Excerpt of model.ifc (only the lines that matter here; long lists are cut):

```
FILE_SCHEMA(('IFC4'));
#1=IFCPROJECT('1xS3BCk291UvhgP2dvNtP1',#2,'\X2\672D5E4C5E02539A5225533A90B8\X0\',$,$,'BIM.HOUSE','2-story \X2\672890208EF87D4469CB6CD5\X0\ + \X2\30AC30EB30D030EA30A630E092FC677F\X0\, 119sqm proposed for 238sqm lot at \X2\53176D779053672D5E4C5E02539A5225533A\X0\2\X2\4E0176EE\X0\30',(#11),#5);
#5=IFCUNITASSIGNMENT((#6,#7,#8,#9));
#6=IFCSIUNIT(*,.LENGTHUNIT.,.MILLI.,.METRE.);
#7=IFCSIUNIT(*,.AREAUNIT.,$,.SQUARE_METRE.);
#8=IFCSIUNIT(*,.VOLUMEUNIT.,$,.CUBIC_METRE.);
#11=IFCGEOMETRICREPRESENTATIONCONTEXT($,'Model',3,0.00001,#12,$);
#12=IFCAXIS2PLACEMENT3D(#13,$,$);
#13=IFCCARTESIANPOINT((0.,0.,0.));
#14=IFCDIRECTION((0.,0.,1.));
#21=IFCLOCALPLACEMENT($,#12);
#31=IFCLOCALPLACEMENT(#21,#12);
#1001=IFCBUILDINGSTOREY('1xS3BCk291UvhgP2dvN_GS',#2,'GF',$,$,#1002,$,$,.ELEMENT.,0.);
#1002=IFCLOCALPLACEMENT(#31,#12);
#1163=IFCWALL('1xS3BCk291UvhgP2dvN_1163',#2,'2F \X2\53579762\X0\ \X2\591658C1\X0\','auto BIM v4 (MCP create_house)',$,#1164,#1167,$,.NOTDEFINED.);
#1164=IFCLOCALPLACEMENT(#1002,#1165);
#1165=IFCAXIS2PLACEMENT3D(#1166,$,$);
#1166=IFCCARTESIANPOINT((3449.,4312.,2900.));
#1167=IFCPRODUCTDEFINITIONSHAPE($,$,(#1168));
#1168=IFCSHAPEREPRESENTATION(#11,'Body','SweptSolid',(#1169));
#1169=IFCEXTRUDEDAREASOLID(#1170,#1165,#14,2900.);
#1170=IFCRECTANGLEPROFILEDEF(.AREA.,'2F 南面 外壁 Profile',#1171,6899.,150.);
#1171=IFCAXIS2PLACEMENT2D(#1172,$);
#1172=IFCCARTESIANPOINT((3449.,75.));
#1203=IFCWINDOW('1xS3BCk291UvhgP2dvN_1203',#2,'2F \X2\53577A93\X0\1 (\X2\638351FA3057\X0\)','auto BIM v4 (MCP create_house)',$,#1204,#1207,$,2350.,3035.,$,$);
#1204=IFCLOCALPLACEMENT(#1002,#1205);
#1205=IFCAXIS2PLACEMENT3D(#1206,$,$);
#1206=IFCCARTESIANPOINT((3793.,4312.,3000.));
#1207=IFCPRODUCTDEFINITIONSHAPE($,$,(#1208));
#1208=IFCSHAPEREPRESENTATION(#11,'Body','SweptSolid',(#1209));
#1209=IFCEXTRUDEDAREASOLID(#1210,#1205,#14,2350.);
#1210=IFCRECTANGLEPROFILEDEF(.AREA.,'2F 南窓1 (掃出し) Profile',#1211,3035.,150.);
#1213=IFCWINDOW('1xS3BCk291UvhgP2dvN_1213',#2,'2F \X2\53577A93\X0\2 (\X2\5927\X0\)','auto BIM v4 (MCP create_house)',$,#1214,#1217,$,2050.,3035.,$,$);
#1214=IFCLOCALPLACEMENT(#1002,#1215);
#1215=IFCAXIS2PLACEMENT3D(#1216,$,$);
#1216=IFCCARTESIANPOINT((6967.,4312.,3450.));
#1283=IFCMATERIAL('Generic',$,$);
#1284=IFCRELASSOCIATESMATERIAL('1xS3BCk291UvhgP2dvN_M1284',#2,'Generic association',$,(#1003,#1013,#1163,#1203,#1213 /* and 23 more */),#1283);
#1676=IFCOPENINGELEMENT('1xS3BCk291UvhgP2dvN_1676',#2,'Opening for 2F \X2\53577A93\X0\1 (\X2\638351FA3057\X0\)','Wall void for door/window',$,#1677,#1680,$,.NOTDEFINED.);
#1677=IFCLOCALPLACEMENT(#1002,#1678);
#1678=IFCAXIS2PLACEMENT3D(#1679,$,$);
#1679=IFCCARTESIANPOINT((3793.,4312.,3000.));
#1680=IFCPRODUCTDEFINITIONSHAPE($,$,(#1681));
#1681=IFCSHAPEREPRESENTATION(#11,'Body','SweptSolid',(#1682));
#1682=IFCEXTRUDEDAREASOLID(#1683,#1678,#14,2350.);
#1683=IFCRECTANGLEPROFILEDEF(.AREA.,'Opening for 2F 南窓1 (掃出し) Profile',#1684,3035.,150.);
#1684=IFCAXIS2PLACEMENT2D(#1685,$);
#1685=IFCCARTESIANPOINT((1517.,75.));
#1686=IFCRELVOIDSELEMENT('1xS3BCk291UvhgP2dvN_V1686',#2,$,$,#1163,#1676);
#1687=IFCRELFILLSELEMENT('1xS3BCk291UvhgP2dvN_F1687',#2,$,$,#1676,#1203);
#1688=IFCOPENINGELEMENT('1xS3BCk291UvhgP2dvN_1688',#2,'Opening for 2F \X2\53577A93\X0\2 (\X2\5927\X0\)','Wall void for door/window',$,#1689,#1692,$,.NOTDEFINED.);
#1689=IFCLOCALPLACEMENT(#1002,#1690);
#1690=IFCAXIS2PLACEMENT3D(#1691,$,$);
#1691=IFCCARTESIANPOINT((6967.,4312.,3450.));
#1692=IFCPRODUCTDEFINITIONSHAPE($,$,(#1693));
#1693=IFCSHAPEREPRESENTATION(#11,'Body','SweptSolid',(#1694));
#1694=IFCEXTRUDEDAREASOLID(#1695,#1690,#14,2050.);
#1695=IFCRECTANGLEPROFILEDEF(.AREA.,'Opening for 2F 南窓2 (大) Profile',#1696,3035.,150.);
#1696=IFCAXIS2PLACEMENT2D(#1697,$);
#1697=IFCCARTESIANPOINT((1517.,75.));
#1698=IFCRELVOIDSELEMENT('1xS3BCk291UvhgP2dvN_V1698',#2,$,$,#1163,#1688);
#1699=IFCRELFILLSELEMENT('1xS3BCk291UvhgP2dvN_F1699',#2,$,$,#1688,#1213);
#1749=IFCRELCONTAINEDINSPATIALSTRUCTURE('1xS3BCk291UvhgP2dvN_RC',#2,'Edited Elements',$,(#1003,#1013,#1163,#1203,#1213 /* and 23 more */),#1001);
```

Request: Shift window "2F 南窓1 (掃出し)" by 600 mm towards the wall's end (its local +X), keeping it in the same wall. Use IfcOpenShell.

```python
import ifcopenshell
import ifcopenshell.api.geometry
import ifcopenshell.util.placement
import ifcopenshell.util.unit

model = ifcopenshell.open("model.ifc")
unit_scale = ifcopenshell.util.unit.calculate_unit_scale(model)

window = model.by_guid("1xS3BCk291UvhgP2dvN_1203")
opening = window.FillsVoids[0].RelatingOpeningElement
wall = opening.VoidsElements[0].RelatingBuildingElement

wall_matrix = ifcopenshell.util.placement.get_local_placement(wall.ObjectPlacement)
shift = wall_matrix[:3, 0] * 0.6 / unit_scale
before = ifcopenshell.util.placement.get_local_placement(window.ObjectPlacement)[:3, 3].copy()

# The window is not placed relative to its opening, so move both.
for product in (opening, window):
    matrix = ifcopenshell.util.placement.get_local_placement(product.ObjectPlacement)
    matrix[:3, 3] += shift
    ifcopenshell.api.geometry.edit_object_placement(model, product=product, matrix=matrix, is_si=False)

after = ifcopenshell.util.placement.get_local_placement(window.ObjectPlacement)[:3, 3]
print("window moved by", (after - before).round(3) + 0.0)

model.write("model-out.ifc")
```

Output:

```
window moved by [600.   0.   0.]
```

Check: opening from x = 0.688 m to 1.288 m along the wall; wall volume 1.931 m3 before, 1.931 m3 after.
